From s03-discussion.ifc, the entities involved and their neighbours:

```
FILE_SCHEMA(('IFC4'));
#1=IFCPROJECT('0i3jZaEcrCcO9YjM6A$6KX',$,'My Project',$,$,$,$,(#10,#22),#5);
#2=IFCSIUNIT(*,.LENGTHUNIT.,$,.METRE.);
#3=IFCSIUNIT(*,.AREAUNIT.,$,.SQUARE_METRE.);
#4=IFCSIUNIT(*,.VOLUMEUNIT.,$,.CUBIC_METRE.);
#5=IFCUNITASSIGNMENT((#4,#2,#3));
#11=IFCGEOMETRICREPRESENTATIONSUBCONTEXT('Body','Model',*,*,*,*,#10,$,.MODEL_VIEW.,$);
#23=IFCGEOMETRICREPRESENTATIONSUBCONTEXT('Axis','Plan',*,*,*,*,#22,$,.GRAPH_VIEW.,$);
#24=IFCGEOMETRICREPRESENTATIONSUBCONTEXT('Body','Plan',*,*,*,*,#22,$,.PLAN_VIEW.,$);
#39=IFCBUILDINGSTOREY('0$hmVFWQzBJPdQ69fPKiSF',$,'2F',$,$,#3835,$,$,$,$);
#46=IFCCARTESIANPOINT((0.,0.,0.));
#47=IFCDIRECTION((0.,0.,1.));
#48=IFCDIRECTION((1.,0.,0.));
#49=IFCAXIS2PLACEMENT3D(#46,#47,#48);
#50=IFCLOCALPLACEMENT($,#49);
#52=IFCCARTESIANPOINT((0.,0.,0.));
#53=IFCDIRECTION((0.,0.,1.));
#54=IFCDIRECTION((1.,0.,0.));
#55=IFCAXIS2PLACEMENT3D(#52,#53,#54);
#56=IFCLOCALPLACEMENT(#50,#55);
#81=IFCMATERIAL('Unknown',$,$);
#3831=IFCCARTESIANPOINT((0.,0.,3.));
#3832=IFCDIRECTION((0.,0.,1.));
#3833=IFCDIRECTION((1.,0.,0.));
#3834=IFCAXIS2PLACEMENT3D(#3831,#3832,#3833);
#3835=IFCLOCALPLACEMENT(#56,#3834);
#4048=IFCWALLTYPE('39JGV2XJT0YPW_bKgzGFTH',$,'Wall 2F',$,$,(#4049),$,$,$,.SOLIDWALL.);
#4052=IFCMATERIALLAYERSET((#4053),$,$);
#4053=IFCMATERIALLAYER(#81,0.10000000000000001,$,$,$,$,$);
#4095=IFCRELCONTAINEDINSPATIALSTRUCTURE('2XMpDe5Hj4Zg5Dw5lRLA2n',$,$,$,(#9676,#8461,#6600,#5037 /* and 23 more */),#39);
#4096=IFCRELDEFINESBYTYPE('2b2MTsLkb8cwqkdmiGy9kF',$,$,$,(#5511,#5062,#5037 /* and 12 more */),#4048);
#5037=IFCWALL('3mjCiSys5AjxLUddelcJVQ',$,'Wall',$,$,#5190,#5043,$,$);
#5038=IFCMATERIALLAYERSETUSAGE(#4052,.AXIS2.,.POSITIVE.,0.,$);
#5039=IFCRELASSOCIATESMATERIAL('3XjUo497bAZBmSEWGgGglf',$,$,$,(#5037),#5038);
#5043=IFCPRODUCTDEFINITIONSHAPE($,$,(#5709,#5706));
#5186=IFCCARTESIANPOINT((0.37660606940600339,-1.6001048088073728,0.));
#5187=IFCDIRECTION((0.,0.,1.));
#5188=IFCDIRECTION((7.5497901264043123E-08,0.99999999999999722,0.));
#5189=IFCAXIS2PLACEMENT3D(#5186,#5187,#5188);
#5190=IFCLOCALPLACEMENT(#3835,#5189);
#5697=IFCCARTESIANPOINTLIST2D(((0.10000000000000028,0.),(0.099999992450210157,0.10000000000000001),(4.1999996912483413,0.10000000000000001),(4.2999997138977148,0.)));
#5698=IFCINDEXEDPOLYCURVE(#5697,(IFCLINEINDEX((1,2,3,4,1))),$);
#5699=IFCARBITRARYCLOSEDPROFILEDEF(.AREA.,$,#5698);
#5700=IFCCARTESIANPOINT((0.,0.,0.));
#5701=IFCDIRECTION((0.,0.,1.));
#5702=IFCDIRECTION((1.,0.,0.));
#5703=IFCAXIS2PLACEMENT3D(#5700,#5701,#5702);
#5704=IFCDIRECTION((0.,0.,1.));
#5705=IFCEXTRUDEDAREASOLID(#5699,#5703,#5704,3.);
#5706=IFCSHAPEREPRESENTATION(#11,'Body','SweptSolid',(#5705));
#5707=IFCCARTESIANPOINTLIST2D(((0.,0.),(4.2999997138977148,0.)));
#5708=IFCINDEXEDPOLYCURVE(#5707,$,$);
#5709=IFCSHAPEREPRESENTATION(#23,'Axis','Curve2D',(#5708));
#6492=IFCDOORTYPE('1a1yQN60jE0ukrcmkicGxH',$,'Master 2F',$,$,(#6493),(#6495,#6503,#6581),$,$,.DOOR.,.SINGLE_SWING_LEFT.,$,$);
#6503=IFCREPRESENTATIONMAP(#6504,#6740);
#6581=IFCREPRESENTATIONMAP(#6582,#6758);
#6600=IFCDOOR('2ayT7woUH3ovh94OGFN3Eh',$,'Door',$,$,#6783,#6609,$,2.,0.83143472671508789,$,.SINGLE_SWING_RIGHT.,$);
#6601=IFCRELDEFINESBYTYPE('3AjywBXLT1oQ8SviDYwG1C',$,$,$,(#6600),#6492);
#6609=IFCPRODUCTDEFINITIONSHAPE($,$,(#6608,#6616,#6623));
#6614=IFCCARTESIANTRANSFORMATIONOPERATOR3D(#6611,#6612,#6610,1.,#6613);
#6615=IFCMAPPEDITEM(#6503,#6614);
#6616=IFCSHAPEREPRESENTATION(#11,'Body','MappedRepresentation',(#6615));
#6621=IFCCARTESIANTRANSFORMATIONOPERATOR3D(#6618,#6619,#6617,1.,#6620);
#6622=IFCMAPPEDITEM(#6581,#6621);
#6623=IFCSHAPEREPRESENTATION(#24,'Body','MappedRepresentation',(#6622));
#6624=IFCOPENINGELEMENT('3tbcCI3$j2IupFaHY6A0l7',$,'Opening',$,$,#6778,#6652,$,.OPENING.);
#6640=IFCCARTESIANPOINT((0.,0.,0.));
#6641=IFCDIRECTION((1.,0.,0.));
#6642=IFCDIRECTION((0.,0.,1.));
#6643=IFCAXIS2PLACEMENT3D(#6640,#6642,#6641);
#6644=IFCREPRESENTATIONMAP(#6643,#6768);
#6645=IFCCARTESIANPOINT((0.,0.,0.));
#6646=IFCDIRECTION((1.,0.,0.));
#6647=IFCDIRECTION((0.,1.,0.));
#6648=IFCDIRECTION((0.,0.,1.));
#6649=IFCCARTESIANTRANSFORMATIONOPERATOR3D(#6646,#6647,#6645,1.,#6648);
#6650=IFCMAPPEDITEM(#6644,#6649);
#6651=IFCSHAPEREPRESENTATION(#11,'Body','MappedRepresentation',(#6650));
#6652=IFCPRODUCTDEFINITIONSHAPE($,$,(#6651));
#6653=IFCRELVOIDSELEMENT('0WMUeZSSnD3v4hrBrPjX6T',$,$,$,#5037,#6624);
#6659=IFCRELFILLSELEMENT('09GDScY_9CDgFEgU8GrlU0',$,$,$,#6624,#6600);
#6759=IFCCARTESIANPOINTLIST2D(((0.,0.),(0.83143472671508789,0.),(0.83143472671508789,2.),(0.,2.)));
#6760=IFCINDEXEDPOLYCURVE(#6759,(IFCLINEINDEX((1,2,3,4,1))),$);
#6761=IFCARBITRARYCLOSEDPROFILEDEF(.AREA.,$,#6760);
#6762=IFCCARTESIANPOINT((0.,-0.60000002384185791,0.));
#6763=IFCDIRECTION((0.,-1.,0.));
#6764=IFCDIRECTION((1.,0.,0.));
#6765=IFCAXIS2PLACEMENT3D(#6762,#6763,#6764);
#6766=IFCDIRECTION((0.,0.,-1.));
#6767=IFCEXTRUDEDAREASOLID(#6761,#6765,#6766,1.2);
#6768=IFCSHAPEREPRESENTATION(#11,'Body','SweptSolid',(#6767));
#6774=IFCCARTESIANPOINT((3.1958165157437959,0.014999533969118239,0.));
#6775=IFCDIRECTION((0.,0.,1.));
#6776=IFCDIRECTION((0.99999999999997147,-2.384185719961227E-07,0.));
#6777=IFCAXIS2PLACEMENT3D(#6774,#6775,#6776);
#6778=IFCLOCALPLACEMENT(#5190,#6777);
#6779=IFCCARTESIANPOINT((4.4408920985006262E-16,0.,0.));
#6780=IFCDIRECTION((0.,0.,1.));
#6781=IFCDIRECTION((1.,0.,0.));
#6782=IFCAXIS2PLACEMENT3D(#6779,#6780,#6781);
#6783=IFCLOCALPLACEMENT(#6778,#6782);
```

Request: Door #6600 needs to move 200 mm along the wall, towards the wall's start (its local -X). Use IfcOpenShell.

```python
import ifcopenshell
import ifcopenshell.api.geometry
import ifcopenshell.util.placement
import ifcopenshell.util.unit

model = ifcopenshell.open("s03-discussion.ifc")
unit_scale = ifcopenshell.util.unit.calculate_unit_scale(model)

door = model.by_guid("2ayT7woUH3ovh94OGFN3Eh")
opening = door.FillsVoids[0].RelatingOpeningElement
wall = opening.VoidsElements[0].RelatingBuildingElement

wall_matrix = ifcopenshell.util.placement.get_local_placement(wall.ObjectPlacement)
shift = wall_matrix[:3, 0] * -0.2 / unit_scale
before = ifcopenshell.util.placement.get_local_placement(door.ObjectPlacement)[:3, 3].copy()

# The door is placed relative to its opening, so it follows when the opening moves.
matrix = ifcopenshell.util.placement.get_local_placement(opening.ObjectPlacement)
matrix[:3, 3] += shift
ifcopenshell.api.geometry.edit_object_placement(
    model, product=opening, matrix=matrix, is_si=False, should_transform_children=True
)

after = ifcopenshell.util.placement.get_local_placement(door.ObjectPlacement)[:3, 3]
print("door moved by", (after - before).round(3) + 0.0)

model.write("s03-discussion_edited.ifc")
```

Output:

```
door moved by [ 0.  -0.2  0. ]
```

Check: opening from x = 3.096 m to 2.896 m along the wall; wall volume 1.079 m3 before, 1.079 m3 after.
